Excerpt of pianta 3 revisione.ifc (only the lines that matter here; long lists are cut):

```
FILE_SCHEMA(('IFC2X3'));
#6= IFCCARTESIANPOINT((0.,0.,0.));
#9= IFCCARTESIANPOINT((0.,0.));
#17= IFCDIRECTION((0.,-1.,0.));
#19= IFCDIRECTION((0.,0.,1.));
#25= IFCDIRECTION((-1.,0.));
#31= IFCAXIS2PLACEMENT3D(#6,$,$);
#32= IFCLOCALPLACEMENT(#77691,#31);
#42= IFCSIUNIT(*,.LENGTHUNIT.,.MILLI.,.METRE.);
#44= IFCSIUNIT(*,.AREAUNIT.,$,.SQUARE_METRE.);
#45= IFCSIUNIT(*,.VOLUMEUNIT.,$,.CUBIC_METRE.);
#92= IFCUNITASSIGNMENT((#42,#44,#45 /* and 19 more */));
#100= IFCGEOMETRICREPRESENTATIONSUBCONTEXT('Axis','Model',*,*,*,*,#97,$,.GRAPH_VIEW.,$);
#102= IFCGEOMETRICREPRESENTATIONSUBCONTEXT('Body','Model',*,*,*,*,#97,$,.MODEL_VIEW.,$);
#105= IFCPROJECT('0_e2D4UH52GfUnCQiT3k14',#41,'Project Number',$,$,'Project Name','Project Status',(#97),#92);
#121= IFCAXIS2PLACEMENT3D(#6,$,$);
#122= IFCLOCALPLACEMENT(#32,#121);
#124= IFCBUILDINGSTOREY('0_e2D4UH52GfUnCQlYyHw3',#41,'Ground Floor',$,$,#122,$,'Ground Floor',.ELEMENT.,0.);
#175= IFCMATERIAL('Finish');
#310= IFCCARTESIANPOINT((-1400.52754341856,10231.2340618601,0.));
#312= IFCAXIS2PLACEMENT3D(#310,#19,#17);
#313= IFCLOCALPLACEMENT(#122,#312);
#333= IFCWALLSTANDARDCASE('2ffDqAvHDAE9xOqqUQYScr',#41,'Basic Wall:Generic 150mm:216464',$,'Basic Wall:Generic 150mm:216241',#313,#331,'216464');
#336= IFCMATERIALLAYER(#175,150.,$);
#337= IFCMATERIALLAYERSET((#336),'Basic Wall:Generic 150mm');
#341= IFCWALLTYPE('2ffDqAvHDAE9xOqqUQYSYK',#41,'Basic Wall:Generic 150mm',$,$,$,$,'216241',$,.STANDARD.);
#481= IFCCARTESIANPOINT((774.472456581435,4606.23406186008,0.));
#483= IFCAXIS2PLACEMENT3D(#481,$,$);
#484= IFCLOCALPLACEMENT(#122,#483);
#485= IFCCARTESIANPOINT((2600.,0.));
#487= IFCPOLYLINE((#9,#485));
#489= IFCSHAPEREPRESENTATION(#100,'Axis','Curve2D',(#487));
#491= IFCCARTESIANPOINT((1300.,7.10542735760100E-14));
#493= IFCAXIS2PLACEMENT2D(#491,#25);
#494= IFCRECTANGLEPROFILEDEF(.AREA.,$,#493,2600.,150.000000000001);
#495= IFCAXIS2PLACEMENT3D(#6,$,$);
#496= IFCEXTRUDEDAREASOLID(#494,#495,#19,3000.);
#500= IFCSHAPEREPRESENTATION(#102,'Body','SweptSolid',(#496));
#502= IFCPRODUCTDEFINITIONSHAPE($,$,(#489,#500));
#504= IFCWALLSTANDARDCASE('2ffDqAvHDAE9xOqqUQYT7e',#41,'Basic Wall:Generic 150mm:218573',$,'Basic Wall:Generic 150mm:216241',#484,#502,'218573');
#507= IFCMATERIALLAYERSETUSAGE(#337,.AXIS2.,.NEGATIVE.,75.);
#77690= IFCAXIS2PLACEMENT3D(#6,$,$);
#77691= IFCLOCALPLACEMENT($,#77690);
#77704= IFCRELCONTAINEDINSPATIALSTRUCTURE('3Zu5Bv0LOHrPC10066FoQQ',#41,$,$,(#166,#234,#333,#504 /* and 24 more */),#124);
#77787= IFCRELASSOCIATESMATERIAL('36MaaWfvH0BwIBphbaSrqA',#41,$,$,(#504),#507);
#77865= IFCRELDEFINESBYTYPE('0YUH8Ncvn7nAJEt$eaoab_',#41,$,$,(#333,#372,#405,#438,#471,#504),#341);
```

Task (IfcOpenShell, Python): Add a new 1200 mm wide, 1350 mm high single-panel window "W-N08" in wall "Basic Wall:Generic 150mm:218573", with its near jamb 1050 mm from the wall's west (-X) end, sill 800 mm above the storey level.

```python
import numpy as np
import ifcopenshell
import ifcopenshell.api.feature
import ifcopenshell.api.geometry
import ifcopenshell.api.root
import ifcopenshell.api.spatial
import ifcopenshell.api.type
import ifcopenshell.geom
import ifcopenshell.util.element
import ifcopenshell.util.placement
import ifcopenshell.util.representation
import ifcopenshell.util.shape
import ifcopenshell.util.unit

model = ifcopenshell.open("pianta 3 revisione.ifc")
unit_scale = ifcopenshell.util.unit.calculate_unit_scale(model)
settings = ifcopenshell.geom.settings()


def volume(element):
    """Net volume in cubic metres, openings subtracted."""
    shape = ifcopenshell.geom.create_shape(settings, element)
    return ifcopenshell.util.shape.get_volume(shape.geometry)


wall = model.by_guid("2ffDqAvHDAE9xOqqUQYT7e")
storey = ifcopenshell.util.element.get_container(wall, ifc_class="IfcBuildingStorey")
context = ifcopenshell.util.representation.get_context(model, "Model", "Body", "MODEL_VIEW")
before = volume(wall)

width, height, from_end, sill = 1.2, 1.35, 1.05, 0.8  # metres

# The wall runs along its own X axis, and the end named is its -X end.
wall_shape = ifcopenshell.geom.create_shape(settings, wall)
x, y, z = ifcopenshell.util.shape.get_vertices(wall_shape.geometry).T
start = x.min() + from_end
face, thickness = float(y.min()), float(y.max() - y.min())
wall_matrix = ifcopenshell.util.placement.get_local_placement(wall.ObjectPlacement)
level = ifcopenshell.util.placement.get_local_placement(storey.ObjectPlacement)[2, 3]


def in_wall(x, y):
    """Placement at x, y metres in the wall's axes, at sill height."""
    matrix = wall_matrix.copy()
    matrix[:, 3] = wall_matrix @ np.array([x / unit_scale, y / unit_scale, 0.0, 1.0])
    matrix[2, 3] = level + sill / unit_scale
    return matrix


# Opening: a box that overshoots both wall faces by 50 mm.
opening = ifcopenshell.api.root.create_entity(model, ifc_class="IfcOpeningElement")
box = ifcopenshell.api.geometry.add_wall_representation(
    model, context=context, length=width, height=height, thickness=thickness + 0.1
)
ifcopenshell.api.geometry.assign_representation(model, product=opening, representation=box)
ifcopenshell.api.geometry.edit_object_placement(model, product=opening, matrix=in_wall(start, face - 0.05), is_si=False)
ifcopenshell.api.feature.add_feature(model, feature=opening, element=wall)

window = ifcopenshell.api.root.create_entity(model, ifc_class="IfcWindow", name="W-N08")
window.OverallWidth, window.OverallHeight = width / unit_scale, height / unit_scale
body = ifcopenshell.api.geometry.add_window_representation(
    model,
    context=context,
    overall_width=window.OverallWidth,
    overall_height=window.OverallHeight,
    partition_type="SINGLE_PANEL",
)
ifcopenshell.api.geometry.assign_representation(model, product=window, representation=body)
ifcopenshell.api.spatial.assign_container(model, products=[window], relating_structure=storey)
fills = ifcopenshell.api.feature.add_filling(model, opening=opening, element=window)
fills.OwnerHistory = window.OwnerHistory  # required in IFC2X3

# IFC2X3 keeps the operation on the window style.
style = ifcopenshell.api.root.create_entity(model, ifc_class="IfcWindowStyle", name="W-N08")
style.OperationType, style.ConstructionType = "SINGLE_PANEL", "NOTDEFINED"
style.ParameterTakesPrecedence = style.Sizeable = False
ifcopenshell.api.type.assign_type(model, related_objects=[window], relating_type=style)

# Centre the window in the wall's thickness.
ifcopenshell.api.geometry.edit_object_placement(model, product=window, matrix=in_wall(start, face), is_si=False)
window_shape = ifcopenshell.geom.create_shape(settings, window)
depth = ifcopenshell.util.shape.get_vertices(window_shape.geometry)[:, 1]
offset = face + thickness / 2 - (depth.min() + depth.max()) / 2
ifcopenshell.api.geometry.edit_object_placement(model, product=window, matrix=in_wall(start, offset), is_si=False)

after = volume(wall)

print(f"wall volume {before:.3f} -> {after:.3f} m3")

model.write("pianta 3 revisione_updated.ifc")
```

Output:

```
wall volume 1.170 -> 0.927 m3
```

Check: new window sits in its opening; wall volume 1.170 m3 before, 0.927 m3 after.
